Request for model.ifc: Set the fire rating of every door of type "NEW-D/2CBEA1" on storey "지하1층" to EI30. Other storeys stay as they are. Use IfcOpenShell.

First a look at what the model holds.

```python
import ifcopenshell
import ifcopenshell.util.element

model = ifcopenshell.open("model.ifc")
print(model.schema)
storey = next(s for s in model.by_type("IfcBuildingStorey") if s.Name == "지하1층")
doors = [e for e in ifcopenshell.util.element.get_decomposition(storey) if e.is_a("IfcDoor")]
seen = {}
for e in doors:
    element_type = ifcopenshell.util.element.get_type(e)
    key = (element_type.Name if element_type != e and element_type else None, ifcopenshell.util.element.get_pset(e, "Pset_DoorCommon", "FireRating"))
    seen[key] = seen.get(key, 0) + 1
for (name, value), count in sorted(seen.items(), key=str):
    print(count, "x", name, "|", value)
```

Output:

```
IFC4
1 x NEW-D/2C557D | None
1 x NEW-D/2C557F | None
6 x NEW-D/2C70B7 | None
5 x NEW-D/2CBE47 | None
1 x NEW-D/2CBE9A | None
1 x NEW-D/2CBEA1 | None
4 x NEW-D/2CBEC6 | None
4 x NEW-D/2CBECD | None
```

```python
import ifcopenshell
import ifcopenshell.api.pset
import ifcopenshell.util.element

model = ifcopenshell.open("model.ifc")

storey = next(s for s in model.by_type("IfcBuildingStorey") if s.Name == "지하1층")
doors = [e for e in ifcopenshell.util.element.get_decomposition(storey) if e.is_a("IfcDoor")]

count = 0
for e in doors:
    element_type = ifcopenshell.util.element.get_type(e)
    if element_type in (None, e) or element_type.Name != "NEW-D/2CBEA1":
        continue
    # add_pset returns the element's existing set when there is one.
    pset = ifcopenshell.api.pset.add_pset(model, product=e, name="Pset_DoorCommon")
    ifcopenshell.api.pset.edit_pset(model, pset=pset, properties={"FireRating": "EI30"})
    count += 1

print(count, "doors updated")

model.write("model_updated.ifc")
```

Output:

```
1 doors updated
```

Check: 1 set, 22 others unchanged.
